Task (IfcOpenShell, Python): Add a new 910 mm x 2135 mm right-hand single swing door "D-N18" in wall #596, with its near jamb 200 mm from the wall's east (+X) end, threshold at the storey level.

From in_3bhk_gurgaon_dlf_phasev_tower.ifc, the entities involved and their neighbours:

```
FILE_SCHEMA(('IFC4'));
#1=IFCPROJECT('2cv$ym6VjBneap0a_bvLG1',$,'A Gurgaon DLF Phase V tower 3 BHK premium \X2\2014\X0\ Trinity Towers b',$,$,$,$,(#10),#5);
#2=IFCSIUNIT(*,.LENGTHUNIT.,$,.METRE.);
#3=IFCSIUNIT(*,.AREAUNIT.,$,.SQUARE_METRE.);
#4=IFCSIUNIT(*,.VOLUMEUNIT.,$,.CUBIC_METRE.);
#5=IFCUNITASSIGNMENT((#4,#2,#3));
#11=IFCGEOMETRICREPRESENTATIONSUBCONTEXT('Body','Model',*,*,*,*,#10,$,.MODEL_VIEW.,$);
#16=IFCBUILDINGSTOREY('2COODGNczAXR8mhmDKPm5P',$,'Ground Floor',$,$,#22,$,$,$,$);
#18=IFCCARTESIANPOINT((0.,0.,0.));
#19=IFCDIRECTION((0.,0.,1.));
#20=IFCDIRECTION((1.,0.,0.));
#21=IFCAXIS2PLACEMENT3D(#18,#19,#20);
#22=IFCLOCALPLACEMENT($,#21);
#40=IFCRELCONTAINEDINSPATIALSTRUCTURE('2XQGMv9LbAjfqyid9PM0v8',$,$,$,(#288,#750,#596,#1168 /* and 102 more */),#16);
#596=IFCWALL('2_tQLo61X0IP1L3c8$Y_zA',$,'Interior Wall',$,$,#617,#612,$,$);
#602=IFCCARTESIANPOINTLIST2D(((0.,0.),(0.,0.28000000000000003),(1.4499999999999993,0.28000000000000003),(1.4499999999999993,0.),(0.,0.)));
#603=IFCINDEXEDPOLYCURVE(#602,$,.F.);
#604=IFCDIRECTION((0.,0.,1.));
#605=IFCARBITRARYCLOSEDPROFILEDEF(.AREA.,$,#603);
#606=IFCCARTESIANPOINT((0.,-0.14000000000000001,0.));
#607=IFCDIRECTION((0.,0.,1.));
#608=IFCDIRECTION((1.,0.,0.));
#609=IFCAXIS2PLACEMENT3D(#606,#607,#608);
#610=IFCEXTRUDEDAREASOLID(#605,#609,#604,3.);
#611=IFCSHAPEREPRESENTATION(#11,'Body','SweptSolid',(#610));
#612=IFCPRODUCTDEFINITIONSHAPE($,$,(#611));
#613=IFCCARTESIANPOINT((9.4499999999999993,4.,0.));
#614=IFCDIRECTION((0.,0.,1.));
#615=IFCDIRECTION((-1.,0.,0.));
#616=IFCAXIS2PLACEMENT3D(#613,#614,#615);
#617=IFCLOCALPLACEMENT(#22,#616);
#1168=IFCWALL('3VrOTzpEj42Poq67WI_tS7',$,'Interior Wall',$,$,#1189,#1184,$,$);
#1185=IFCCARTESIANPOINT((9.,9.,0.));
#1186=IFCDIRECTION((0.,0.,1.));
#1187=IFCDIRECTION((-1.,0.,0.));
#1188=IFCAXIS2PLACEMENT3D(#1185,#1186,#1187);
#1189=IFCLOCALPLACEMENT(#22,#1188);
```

```python
import numpy as np
import ifcopenshell
import ifcopenshell.api.feature
import ifcopenshell.api.geometry
import ifcopenshell.api.root
import ifcopenshell.api.spatial
import ifcopenshell.geom
import ifcopenshell.util.element
import ifcopenshell.util.placement
import ifcopenshell.util.representation
import ifcopenshell.util.shape
import ifcopenshell.util.unit

model = ifcopenshell.open("in_3bhk_gurgaon_dlf_phasev_tower.ifc")
unit_scale = ifcopenshell.util.unit.calculate_unit_scale(model)
settings = ifcopenshell.geom.settings()


def volume(element):
    """Net volume in cubic metres, openings subtracted."""
    shape = ifcopenshell.geom.create_shape(settings, element)
    return ifcopenshell.util.shape.get_volume(shape.geometry)


wall = model.by_id(596)
storey = ifcopenshell.util.element.get_container(wall, ifc_class="IfcBuildingStorey")
context = ifcopenshell.util.representation.get_context(model, "Model", "Body", "MODEL_VIEW")
before = volume(wall)

width, height, from_end, sill = 0.91, 2.135, 0.2, 0.0  # metres

# The wall runs along its own X axis, and the end named is its -X end.
wall_shape = ifcopenshell.geom.create_shape(settings, wall)
x, y, z = ifcopenshell.util.shape.get_vertices(wall_shape.geometry).T
start = x.min() + from_end
face, thickness = float(y.min()), float(y.max() - y.min())
wall_matrix = ifcopenshell.util.placement.get_local_placement(wall.ObjectPlacement)
level = ifcopenshell.util.placement.get_local_placement(storey.ObjectPlacement)[2, 3]


def in_wall(x, y):
    """Placement at x, y metres in the wall's axes, at sill height."""
    matrix = wall_matrix.copy()
    matrix[:, 3] = wall_matrix @ np.array([x / unit_scale, y / unit_scale, 0.0, 1.0])
    matrix[2, 3] = level + sill / unit_scale
    return matrix


# Opening: a box that overshoots both wall faces by 50 mm.
opening = ifcopenshell.api.root.create_entity(model, ifc_class="IfcOpeningElement", predefined_type="OPENING")
box = ifcopenshell.api.geometry.add_wall_representation(
    model, context=context, length=width, height=height, thickness=thickness + 0.1
)
ifcopenshell.api.geometry.assign_representation(model, product=opening, representation=box)
ifcopenshell.api.geometry.edit_object_placement(model, product=opening, matrix=in_wall(start, face - 0.05), is_si=False)
ifcopenshell.api.feature.add_feature(model, feature=opening, element=wall)

door = ifcopenshell.api.root.create_entity(model, ifc_class="IfcDoor", name="D-N18", predefined_type="DOOR")
door.OverallWidth, door.OverallHeight = width / unit_scale, height / unit_scale
door.OperationType = "SINGLE_SWING_RIGHT"
body = ifcopenshell.api.geometry.add_door_representation(
    model,
    context=context,
    overall_width=door.OverallWidth,
    overall_height=door.OverallHeight,
    operation_type="SINGLE_SWING_RIGHT",
    lining_properties={"LiningDepth": thickness / unit_scale, "ThresholdDepth": thickness / unit_scale},
)
ifcopenshell.api.geometry.assign_representation(model, product=door, representation=body)
ifcopenshell.api.spatial.assign_container(model, products=[door], relating_structure=storey)
ifcopenshell.api.feature.add_filling(model, opening=opening, element=door)

# The lining spans the wall, so the door starts at the wall face.
ifcopenshell.api.geometry.edit_object_placement(model, product=door, matrix=in_wall(start, face), is_si=False)

after = volume(wall)

print(f"wall volume {before:.3f} -> {after:.3f} m3")

model.write("in_3bhk_gurgaon_dlf_phasev_tower_edited.ifc")
```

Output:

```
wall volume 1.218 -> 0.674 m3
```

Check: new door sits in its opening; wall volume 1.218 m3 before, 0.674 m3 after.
